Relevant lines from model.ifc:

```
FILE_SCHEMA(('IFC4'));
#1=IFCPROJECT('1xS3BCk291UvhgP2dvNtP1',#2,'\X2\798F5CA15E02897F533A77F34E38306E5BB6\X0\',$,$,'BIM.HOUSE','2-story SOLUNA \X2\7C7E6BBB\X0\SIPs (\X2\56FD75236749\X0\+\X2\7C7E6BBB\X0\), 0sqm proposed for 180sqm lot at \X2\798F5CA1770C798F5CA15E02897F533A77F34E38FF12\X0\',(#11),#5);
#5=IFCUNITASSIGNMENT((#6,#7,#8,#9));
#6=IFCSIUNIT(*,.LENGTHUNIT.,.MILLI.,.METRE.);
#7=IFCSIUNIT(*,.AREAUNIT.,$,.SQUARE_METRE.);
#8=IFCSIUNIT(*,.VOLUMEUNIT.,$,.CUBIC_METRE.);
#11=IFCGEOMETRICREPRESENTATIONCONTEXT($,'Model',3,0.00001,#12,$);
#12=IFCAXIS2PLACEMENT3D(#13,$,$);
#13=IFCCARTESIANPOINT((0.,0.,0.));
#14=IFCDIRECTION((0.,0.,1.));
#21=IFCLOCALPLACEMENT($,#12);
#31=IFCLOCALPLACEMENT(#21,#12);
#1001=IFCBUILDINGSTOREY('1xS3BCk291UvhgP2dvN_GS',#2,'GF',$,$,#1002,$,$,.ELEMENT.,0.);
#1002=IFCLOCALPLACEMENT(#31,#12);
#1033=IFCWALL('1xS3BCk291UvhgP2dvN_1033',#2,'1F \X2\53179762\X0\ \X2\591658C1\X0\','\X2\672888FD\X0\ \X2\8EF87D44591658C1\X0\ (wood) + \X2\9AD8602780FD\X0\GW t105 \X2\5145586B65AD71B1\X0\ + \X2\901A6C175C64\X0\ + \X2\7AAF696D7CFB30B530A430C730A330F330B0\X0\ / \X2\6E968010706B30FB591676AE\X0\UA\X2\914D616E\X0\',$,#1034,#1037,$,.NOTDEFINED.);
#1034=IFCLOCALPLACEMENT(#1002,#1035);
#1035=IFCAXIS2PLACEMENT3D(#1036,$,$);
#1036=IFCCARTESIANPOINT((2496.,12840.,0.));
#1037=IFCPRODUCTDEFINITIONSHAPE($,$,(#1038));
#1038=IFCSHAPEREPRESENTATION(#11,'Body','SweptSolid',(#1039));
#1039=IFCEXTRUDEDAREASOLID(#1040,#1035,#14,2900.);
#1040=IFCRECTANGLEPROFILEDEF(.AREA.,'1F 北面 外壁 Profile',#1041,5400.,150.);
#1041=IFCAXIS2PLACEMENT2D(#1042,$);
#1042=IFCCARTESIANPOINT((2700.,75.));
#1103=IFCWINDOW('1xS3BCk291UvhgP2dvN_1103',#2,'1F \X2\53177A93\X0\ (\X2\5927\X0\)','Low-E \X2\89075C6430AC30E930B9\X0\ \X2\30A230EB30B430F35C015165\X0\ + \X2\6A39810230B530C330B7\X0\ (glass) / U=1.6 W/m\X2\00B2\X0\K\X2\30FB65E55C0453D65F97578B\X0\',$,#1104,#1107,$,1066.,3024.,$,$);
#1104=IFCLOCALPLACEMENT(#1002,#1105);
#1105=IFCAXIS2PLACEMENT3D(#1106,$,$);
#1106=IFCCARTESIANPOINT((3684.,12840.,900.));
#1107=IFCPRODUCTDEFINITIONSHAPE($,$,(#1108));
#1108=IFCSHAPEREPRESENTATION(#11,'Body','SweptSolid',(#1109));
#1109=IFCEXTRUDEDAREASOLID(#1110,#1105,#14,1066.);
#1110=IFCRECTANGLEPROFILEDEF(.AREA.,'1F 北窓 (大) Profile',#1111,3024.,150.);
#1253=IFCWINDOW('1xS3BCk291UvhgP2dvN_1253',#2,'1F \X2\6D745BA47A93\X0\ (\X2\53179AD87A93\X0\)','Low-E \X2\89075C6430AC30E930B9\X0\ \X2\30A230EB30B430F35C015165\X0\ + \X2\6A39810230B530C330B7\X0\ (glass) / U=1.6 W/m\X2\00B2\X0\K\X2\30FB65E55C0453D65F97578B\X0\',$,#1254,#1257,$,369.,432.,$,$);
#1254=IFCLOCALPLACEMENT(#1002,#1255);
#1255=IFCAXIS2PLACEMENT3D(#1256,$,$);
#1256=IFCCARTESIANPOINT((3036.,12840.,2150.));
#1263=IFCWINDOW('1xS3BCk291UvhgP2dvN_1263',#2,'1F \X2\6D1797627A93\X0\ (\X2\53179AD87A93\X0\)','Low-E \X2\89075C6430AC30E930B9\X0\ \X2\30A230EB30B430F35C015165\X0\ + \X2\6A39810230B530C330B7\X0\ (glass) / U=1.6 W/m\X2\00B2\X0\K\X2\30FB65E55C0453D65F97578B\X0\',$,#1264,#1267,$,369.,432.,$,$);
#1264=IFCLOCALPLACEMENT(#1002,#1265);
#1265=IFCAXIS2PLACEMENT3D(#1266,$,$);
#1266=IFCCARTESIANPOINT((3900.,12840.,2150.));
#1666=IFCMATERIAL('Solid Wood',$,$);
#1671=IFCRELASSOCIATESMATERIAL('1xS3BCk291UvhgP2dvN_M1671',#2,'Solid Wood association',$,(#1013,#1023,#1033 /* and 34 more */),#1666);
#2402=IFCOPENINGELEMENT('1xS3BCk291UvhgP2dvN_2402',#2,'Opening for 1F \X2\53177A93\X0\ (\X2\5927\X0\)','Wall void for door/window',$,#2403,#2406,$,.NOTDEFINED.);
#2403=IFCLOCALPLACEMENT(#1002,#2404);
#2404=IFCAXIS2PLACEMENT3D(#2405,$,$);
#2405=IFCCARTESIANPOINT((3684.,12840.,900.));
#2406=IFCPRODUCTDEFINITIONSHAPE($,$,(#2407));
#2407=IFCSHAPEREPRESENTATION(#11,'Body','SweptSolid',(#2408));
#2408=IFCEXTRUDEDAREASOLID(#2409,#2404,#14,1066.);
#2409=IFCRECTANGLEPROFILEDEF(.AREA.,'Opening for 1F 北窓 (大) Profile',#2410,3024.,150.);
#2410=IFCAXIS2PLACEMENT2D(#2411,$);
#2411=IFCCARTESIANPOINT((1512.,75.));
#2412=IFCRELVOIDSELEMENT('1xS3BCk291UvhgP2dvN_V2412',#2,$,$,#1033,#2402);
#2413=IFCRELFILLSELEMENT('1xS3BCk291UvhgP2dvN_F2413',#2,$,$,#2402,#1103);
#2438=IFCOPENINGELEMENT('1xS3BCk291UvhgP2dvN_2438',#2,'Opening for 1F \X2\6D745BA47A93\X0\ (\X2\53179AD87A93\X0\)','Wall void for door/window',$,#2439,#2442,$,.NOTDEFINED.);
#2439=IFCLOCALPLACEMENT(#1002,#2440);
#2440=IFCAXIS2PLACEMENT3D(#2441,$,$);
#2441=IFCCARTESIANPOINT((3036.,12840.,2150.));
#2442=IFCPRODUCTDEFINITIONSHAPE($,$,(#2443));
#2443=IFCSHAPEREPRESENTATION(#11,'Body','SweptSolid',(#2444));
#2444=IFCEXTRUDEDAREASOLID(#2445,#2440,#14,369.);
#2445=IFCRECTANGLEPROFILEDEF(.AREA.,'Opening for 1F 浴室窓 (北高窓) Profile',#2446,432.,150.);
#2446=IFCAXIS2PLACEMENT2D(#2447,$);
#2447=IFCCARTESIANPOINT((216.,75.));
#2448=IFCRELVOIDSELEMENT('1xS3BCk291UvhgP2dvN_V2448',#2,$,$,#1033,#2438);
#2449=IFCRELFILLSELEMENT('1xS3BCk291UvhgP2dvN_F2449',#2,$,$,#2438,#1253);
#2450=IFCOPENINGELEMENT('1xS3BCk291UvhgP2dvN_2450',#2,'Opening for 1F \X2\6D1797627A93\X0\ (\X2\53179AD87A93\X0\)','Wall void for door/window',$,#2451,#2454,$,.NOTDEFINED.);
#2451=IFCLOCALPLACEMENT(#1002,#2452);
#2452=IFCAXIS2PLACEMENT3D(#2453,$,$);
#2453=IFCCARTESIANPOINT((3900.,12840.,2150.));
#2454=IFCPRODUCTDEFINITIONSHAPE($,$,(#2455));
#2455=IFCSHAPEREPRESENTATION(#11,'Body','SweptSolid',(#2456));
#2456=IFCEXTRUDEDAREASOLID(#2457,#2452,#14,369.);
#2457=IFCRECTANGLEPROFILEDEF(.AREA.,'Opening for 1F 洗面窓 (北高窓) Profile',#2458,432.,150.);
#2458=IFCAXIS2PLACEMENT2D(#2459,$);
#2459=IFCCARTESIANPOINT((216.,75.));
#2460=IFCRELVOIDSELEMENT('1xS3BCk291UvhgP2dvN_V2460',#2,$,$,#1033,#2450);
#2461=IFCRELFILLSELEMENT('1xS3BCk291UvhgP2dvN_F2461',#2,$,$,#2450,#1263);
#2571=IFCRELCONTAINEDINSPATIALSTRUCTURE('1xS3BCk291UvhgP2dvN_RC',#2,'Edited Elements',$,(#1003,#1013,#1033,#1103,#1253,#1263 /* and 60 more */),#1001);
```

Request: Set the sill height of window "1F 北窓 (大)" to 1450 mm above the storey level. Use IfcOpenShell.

```python
import numpy as np
import ifcopenshell
import ifcopenshell.api.geometry
import ifcopenshell.geom
import ifcopenshell.util.element
import ifcopenshell.util.placement
import ifcopenshell.util.shape
import ifcopenshell.util.unit

model = ifcopenshell.open("model.ifc")
unit_scale = ifcopenshell.util.unit.calculate_unit_scale(model)

window = model.by_guid("1xS3BCk291UvhgP2dvN_1103")
opening = window.FillsVoids[0].RelatingOpeningElement
storey = ifcopenshell.util.element.get_container(window, ifc_class="IfcBuildingStorey")
level = ifcopenshell.util.placement.get_local_placement(storey.ObjectPlacement)[2, 3]

# The opening's origin need not be at the sill, so measure its lowest point.
shape = ifcopenshell.geom.create_shape(ifcopenshell.geom.settings(), opening)
bottom = ifcopenshell.util.shape.get_shape_bottom_elevation(shape, shape.geometry) / unit_scale
dz = level + 1450.0 - bottom

shift = np.array([0.0, 0.0, dz])
# The window is not placed relative to its opening, so move both.
for product in (opening, window):
    matrix = ifcopenshell.util.placement.get_local_placement(product.ObjectPlacement)
    matrix[:3, 3] += shift
    ifcopenshell.api.geometry.edit_object_placement(model, product=product, matrix=matrix, is_si=False)

print(f"moved by {dz * unit_scale:+.3f} m")

model.write("model_v2.ifc")
```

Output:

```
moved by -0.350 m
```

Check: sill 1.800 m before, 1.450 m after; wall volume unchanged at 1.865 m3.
